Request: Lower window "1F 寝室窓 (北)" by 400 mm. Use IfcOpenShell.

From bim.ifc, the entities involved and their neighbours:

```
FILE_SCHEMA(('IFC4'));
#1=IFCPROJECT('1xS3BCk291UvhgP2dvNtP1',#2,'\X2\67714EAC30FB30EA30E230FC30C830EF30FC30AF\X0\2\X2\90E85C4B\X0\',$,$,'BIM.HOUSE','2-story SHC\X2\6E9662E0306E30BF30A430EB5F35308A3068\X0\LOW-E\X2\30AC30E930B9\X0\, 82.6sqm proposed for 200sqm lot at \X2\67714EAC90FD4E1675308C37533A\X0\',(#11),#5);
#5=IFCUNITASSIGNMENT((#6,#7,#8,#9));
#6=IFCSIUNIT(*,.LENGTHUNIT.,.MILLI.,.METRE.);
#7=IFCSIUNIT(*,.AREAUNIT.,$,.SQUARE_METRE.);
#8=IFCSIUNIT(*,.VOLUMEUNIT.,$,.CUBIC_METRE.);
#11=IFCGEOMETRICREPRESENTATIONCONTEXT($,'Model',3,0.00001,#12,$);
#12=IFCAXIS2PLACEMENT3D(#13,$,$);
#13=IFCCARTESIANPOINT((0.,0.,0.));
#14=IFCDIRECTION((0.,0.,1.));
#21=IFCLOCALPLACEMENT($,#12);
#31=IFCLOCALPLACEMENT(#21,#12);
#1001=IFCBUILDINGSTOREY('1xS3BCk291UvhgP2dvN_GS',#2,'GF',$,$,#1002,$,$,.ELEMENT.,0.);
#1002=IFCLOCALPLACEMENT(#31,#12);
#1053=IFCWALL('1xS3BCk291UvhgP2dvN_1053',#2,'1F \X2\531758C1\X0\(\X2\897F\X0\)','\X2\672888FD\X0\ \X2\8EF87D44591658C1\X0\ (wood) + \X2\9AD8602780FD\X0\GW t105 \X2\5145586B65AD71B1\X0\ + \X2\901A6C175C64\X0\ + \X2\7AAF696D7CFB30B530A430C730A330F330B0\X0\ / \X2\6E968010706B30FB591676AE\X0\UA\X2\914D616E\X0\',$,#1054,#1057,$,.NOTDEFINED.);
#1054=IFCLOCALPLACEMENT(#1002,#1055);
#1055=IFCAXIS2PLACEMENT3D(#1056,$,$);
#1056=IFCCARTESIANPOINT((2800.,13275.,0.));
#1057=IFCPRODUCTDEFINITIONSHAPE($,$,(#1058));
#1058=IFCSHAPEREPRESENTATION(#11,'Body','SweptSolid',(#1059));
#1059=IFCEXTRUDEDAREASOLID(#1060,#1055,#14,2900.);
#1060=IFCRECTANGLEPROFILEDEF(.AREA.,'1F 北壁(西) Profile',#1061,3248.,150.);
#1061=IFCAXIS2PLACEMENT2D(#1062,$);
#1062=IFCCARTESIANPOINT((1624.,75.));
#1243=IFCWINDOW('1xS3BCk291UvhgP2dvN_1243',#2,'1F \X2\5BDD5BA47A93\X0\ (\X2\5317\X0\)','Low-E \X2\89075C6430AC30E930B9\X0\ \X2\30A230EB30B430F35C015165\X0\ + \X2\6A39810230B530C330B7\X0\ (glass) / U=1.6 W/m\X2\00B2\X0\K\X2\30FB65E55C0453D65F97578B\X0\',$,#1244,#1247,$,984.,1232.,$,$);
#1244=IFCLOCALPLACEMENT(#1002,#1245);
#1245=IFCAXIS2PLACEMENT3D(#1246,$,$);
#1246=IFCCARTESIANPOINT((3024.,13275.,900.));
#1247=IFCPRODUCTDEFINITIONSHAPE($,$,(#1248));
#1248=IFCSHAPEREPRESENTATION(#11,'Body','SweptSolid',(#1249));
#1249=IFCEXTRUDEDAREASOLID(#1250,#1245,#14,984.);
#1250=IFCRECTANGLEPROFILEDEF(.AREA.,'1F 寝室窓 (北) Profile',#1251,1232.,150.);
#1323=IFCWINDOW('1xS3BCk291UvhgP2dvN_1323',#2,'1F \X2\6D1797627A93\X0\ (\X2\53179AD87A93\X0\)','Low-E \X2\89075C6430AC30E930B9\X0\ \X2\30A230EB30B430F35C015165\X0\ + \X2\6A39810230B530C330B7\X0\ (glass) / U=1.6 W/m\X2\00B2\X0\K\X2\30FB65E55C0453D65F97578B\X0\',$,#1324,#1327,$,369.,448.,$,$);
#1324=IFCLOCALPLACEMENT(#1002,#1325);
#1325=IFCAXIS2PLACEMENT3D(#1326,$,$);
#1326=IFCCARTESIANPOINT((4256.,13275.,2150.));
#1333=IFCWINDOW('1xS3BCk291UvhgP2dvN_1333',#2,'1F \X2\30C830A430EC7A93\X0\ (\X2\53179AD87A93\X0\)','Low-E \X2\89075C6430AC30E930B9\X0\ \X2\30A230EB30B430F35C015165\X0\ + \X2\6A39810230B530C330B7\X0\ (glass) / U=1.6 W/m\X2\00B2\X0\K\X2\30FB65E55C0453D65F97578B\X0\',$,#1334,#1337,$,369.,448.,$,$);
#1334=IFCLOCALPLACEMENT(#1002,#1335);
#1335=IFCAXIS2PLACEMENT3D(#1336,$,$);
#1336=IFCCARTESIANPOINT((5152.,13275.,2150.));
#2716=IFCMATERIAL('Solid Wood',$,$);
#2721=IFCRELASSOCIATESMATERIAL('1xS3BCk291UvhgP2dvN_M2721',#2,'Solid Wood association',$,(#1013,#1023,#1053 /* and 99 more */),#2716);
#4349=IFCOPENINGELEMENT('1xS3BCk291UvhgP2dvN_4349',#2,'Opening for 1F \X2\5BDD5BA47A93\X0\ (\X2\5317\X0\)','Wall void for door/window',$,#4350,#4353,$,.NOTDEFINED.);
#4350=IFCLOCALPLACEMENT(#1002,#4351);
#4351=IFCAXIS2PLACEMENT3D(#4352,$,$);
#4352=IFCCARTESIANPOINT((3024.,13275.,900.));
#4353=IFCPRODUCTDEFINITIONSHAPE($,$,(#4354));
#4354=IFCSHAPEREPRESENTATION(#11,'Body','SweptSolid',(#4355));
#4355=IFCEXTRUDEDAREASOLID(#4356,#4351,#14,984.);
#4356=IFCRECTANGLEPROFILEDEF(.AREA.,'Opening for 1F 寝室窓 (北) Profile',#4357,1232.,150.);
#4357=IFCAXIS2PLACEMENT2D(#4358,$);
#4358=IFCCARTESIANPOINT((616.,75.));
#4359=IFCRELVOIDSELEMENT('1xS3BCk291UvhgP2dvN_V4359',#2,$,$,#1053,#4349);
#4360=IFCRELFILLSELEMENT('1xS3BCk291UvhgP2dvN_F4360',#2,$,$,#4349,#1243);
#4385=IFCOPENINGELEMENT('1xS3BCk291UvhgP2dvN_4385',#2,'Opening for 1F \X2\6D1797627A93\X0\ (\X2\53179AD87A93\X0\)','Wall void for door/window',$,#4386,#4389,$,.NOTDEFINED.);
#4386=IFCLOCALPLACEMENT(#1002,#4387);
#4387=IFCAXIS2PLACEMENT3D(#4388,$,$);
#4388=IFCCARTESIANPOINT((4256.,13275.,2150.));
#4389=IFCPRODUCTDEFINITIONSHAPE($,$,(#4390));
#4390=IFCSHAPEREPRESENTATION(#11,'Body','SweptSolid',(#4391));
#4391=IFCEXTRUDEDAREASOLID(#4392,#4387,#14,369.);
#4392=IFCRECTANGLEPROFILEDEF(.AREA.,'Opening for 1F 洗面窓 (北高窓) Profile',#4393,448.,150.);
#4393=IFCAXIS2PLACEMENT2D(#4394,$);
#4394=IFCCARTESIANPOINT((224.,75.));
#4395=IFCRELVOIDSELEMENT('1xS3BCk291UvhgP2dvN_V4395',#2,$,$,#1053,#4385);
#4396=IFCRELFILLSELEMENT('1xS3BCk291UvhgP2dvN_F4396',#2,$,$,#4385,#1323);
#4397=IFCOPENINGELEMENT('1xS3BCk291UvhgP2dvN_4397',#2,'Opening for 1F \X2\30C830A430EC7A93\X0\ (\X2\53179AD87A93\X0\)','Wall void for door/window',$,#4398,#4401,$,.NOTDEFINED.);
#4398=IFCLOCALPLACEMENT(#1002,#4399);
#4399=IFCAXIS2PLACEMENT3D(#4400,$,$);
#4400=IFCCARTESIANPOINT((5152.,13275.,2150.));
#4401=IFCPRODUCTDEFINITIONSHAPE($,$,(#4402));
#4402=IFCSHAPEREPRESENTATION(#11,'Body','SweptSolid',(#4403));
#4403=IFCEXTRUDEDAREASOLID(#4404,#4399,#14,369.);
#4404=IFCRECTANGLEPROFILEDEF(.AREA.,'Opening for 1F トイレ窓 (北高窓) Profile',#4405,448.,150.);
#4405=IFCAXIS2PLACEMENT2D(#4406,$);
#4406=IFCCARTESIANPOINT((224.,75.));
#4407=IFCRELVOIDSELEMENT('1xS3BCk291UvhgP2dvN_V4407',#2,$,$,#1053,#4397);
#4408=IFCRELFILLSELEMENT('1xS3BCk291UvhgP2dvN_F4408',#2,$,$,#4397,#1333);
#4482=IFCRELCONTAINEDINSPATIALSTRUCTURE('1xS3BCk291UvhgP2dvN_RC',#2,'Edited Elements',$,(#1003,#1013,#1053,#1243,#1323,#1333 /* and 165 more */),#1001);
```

```python
import numpy as np
import ifcopenshell
import ifcopenshell.api.geometry
import ifcopenshell.util.placement
import ifcopenshell.util.unit

model = ifcopenshell.open("bim.ifc")
unit_scale = ifcopenshell.util.unit.calculate_unit_scale(model)

window = model.by_guid("1xS3BCk291UvhgP2dvN_1243")
opening = window.FillsVoids[0].RelatingOpeningElement
dz = -400.0

shift = np.array([0.0, 0.0, dz])
# The window is not placed relative to its opening, so move both.
for product in (opening, window):
    matrix = ifcopenshell.util.placement.get_local_placement(product.ObjectPlacement)
    matrix[:3, 3] += shift
    ifcopenshell.api.geometry.edit_object_placement(model, product=product, matrix=matrix, is_si=False)

print(f"moved by {dz * unit_scale:+.3f} m")

model.write("bim_updated.ifc")
```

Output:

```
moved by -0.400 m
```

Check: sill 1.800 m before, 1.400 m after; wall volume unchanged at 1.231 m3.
